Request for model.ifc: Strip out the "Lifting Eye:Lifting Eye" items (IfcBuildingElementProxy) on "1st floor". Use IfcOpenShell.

First a look at what the model holds.

```python
import ifcopenshell
import ifcopenshell.util.element

model = ifcopenshell.open("model.ifc")
print(model.schema)
storey = next(s for s in model.by_type("IfcBuildingStorey") if s.Name == "1st floor")
proxies = [e for e in ifcopenshell.util.element.get_decomposition(storey) if e.is_a("IfcBuildingElementProxy")]
seen = {}
for e in proxies:
    element_type = ifcopenshell.util.element.get_type(e)
    name = element_type.Name if element_type not in (None, e) else None
    seen[name] = seen.get(name, 0) + 1
for name, count in sorted(seen.items(), key=str):
    print(count, "x", name)
```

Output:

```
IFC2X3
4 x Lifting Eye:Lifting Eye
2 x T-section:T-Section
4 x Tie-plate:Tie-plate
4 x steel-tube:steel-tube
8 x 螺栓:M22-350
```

```python
import ifcopenshell
import ifcopenshell.api.root
import ifcopenshell.util.element

model = ifcopenshell.open("model.ifc")

storey = next(s for s in model.by_type("IfcBuildingStorey") if s.Name == "1st floor")
proxies = [e for e in ifcopenshell.util.element.get_decomposition(storey) if e.is_a("IfcBuildingElementProxy")]
targets = [e for e in proxies if (t := ifcopenshell.util.element.get_type(e)) not in (None, e) and t.Name == "Lifting Eye:Lifting Eye"]

for e in targets:
    ifcopenshell.api.root.remove_product(model, product=e)
print(len(targets), "removed")

model.write("model-out.ifc")
```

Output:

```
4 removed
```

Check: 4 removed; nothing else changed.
